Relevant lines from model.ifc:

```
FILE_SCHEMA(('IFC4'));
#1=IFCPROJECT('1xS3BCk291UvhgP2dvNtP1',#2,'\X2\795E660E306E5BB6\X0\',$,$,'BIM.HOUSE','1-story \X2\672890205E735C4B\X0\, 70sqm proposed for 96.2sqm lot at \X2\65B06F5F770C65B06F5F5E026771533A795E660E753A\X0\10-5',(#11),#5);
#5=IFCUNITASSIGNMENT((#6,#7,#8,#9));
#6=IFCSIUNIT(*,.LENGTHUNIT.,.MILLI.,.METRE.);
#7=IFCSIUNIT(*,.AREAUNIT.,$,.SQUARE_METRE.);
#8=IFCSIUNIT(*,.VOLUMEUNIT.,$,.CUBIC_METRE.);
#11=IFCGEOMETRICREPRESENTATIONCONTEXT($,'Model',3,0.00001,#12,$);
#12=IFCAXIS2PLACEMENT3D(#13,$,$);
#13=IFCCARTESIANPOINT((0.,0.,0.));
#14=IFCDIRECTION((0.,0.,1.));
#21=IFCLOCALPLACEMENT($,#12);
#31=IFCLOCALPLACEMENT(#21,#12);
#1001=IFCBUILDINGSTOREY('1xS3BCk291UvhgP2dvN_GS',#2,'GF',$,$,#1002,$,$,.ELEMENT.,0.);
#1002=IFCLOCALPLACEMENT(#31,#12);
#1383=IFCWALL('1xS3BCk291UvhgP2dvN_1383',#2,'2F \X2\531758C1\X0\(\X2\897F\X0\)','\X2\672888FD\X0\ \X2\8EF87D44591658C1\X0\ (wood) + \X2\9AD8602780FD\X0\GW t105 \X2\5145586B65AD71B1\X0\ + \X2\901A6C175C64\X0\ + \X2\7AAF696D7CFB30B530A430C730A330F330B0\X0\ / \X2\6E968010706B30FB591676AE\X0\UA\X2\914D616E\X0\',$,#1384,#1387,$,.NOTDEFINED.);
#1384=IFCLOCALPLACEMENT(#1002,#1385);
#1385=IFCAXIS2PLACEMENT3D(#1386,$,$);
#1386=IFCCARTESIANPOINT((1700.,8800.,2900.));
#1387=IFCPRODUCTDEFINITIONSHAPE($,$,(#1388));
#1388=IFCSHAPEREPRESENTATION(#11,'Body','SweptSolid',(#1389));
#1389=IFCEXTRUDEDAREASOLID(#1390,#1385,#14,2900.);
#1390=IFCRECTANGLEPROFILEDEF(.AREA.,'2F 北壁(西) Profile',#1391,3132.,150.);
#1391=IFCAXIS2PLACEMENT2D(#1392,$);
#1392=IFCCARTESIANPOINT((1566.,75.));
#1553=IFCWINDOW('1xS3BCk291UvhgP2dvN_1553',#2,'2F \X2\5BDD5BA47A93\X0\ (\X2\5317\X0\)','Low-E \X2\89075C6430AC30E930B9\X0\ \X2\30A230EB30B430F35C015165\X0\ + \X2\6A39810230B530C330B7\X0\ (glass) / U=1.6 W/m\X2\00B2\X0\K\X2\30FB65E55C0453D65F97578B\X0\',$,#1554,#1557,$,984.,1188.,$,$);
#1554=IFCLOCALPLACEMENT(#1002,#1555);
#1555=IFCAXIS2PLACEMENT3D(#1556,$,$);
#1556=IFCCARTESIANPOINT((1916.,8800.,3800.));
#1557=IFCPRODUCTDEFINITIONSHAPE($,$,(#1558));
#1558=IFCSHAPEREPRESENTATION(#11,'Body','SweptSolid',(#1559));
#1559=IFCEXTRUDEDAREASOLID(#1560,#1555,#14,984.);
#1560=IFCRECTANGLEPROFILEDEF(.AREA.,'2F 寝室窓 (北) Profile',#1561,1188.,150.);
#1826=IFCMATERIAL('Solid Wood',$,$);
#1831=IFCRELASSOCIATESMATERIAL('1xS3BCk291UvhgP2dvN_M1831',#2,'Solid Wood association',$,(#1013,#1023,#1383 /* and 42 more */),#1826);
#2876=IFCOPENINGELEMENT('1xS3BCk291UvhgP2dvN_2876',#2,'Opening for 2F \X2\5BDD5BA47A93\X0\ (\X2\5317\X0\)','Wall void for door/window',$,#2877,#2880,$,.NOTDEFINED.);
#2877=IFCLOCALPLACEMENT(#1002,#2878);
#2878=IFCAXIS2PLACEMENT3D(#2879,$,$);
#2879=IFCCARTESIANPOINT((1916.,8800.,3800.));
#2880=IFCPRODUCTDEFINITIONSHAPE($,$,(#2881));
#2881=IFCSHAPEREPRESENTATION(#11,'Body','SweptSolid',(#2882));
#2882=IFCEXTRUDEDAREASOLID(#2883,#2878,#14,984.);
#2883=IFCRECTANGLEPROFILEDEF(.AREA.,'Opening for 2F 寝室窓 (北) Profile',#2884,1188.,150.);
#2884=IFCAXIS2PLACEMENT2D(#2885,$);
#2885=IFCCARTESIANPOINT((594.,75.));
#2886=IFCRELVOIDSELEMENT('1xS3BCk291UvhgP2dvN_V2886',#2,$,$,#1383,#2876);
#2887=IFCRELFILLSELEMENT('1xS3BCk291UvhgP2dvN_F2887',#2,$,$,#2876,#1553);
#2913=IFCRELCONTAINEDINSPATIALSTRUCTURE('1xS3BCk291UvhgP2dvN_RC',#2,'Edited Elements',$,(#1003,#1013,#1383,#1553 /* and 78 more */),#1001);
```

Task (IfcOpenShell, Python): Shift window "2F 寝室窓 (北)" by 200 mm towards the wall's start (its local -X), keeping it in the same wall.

```python
import ifcopenshell
import ifcopenshell.api.geometry
import ifcopenshell.util.placement
import ifcopenshell.util.unit

model = ifcopenshell.open("model.ifc")
unit_scale = ifcopenshell.util.unit.calculate_unit_scale(model)

window = model.by_id(1553)
opening = window.FillsVoids[0].RelatingOpeningElement
wall = opening.VoidsElements[0].RelatingBuildingElement

wall_matrix = ifcopenshell.util.placement.get_local_placement(wall.ObjectPlacement)
shift = wall_matrix[:3, 0] * -0.2 / unit_scale
before = ifcopenshell.util.placement.get_local_placement(window.ObjectPlacement)[:3, 3].copy()

# The window is not placed relative to its opening, so move both.
for product in (opening, window):
    matrix = ifcopenshell.util.placement.get_local_placement(product.ObjectPlacement)
    matrix[:3, 3] += shift
    ifcopenshell.api.geometry.edit_object_placement(model, product=product, matrix=matrix, is_si=False)

after = ifcopenshell.util.placement.get_local_placement(window.ObjectPlacement)[:3, 3]
print("window moved by", (after - before).round(3) + 0.0)

model.write("model_rev.ifc")
```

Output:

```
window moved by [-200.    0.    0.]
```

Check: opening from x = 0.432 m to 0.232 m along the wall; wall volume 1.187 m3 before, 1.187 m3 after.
